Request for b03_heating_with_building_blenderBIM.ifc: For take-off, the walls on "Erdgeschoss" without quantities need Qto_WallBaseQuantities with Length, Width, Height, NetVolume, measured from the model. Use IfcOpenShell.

First a look at what the model holds.

```python
import ifcopenshell
import ifcopenshell.util.element
import ifcopenshell.util.unit

model = ifcopenshell.open("b03_heating_with_building_blenderBIM.ifc")
print(model.schema)
for unit_type in ("LENGTHUNIT", "AREAUNIT", "VOLUMEUNIT"):
    print(unit_type, ifcopenshell.util.unit.calculate_unit_scale(model, unit_type))
storey = next(s for s in model.by_type("IfcBuildingStorey") if s.Name == "Erdgeschoss")
walls = [e for e in ifcopenshell.util.element.get_decomposition(storey) if e.is_a("IfcWall")]
for e in sorted(walls, key=lambda e: e.id()):
    print(e.id(), e.is_a(), e.Name, list(ifcopenshell.util.element.get_psets(e, qtos_only=True)), sep=" | ")
```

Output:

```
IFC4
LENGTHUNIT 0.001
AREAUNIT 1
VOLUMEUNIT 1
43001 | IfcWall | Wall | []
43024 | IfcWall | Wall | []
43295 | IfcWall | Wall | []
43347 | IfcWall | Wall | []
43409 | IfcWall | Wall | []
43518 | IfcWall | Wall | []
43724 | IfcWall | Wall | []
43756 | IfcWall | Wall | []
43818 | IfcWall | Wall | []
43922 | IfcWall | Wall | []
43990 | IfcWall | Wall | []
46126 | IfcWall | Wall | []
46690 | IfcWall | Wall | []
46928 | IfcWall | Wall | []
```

```python
import ifcopenshell
import ifcopenshell.api.pset
import ifcopenshell.geom
import ifcopenshell.util.element
import ifcopenshell.util.shape
import ifcopenshell.util.unit

model = ifcopenshell.open("b03_heating_with_building_blenderBIM.ifc")
unit_scale = ifcopenshell.util.unit.calculate_unit_scale(model)
volume_scale = ifcopenshell.util.unit.calculate_unit_scale(model, "VOLUMEUNIT")
settings = ifcopenshell.geom.settings()

storey = next(s for s in model.by_type("IfcBuildingStorey") if s.Name == "Erdgeschoss")
walls = [e for e in ifcopenshell.util.element.get_decomposition(storey) if e.is_a("IfcWall")]

for e in sorted(walls, key=lambda e: e.id()):
    if ifcopenshell.util.element.get_psets(e, qtos_only=True, should_inherit=False):
        continue
    # Geometry comes back in metres, in the element's own axes.
    shape = ifcopenshell.geom.create_shape(settings, e)
    values = {
        "Length": ifcopenshell.util.shape.get_x(shape.geometry) / unit_scale,
        "Width": ifcopenshell.util.shape.get_y(shape.geometry) / unit_scale,
        "Height": ifcopenshell.util.shape.get_z(shape.geometry) / unit_scale,
        "NetVolume": ifcopenshell.util.shape.get_volume(shape.geometry) / volume_scale,
    }
    qto = ifcopenshell.api.pset.add_qto(model, product=e, name="Qto_WallBaseQuantities")
    ifcopenshell.api.pset.edit_qto(model, qto=qto, properties=values)
    print(e.id(), {k: round(v, 3) for k, v in values.items()})

model.write("b03_heating_with_building_blenderBIM_edited.ifc")
```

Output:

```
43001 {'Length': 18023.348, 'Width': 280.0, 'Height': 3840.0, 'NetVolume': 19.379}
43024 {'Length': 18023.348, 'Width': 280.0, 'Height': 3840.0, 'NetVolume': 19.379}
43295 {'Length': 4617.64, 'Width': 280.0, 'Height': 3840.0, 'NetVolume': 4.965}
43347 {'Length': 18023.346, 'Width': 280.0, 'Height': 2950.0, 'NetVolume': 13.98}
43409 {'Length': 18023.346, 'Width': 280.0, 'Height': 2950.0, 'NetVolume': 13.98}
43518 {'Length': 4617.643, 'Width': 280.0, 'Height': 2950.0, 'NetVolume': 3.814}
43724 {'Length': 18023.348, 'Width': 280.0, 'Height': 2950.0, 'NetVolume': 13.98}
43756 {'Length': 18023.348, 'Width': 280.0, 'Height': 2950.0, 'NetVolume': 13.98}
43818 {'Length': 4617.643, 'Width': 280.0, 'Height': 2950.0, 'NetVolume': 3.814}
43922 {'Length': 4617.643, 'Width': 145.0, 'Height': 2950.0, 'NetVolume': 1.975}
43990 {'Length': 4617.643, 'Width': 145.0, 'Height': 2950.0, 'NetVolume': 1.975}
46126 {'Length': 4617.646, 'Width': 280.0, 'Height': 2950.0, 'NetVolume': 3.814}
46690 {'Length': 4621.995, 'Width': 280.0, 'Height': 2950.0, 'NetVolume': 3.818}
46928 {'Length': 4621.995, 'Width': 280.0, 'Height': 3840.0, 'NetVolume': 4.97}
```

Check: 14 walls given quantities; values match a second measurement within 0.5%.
